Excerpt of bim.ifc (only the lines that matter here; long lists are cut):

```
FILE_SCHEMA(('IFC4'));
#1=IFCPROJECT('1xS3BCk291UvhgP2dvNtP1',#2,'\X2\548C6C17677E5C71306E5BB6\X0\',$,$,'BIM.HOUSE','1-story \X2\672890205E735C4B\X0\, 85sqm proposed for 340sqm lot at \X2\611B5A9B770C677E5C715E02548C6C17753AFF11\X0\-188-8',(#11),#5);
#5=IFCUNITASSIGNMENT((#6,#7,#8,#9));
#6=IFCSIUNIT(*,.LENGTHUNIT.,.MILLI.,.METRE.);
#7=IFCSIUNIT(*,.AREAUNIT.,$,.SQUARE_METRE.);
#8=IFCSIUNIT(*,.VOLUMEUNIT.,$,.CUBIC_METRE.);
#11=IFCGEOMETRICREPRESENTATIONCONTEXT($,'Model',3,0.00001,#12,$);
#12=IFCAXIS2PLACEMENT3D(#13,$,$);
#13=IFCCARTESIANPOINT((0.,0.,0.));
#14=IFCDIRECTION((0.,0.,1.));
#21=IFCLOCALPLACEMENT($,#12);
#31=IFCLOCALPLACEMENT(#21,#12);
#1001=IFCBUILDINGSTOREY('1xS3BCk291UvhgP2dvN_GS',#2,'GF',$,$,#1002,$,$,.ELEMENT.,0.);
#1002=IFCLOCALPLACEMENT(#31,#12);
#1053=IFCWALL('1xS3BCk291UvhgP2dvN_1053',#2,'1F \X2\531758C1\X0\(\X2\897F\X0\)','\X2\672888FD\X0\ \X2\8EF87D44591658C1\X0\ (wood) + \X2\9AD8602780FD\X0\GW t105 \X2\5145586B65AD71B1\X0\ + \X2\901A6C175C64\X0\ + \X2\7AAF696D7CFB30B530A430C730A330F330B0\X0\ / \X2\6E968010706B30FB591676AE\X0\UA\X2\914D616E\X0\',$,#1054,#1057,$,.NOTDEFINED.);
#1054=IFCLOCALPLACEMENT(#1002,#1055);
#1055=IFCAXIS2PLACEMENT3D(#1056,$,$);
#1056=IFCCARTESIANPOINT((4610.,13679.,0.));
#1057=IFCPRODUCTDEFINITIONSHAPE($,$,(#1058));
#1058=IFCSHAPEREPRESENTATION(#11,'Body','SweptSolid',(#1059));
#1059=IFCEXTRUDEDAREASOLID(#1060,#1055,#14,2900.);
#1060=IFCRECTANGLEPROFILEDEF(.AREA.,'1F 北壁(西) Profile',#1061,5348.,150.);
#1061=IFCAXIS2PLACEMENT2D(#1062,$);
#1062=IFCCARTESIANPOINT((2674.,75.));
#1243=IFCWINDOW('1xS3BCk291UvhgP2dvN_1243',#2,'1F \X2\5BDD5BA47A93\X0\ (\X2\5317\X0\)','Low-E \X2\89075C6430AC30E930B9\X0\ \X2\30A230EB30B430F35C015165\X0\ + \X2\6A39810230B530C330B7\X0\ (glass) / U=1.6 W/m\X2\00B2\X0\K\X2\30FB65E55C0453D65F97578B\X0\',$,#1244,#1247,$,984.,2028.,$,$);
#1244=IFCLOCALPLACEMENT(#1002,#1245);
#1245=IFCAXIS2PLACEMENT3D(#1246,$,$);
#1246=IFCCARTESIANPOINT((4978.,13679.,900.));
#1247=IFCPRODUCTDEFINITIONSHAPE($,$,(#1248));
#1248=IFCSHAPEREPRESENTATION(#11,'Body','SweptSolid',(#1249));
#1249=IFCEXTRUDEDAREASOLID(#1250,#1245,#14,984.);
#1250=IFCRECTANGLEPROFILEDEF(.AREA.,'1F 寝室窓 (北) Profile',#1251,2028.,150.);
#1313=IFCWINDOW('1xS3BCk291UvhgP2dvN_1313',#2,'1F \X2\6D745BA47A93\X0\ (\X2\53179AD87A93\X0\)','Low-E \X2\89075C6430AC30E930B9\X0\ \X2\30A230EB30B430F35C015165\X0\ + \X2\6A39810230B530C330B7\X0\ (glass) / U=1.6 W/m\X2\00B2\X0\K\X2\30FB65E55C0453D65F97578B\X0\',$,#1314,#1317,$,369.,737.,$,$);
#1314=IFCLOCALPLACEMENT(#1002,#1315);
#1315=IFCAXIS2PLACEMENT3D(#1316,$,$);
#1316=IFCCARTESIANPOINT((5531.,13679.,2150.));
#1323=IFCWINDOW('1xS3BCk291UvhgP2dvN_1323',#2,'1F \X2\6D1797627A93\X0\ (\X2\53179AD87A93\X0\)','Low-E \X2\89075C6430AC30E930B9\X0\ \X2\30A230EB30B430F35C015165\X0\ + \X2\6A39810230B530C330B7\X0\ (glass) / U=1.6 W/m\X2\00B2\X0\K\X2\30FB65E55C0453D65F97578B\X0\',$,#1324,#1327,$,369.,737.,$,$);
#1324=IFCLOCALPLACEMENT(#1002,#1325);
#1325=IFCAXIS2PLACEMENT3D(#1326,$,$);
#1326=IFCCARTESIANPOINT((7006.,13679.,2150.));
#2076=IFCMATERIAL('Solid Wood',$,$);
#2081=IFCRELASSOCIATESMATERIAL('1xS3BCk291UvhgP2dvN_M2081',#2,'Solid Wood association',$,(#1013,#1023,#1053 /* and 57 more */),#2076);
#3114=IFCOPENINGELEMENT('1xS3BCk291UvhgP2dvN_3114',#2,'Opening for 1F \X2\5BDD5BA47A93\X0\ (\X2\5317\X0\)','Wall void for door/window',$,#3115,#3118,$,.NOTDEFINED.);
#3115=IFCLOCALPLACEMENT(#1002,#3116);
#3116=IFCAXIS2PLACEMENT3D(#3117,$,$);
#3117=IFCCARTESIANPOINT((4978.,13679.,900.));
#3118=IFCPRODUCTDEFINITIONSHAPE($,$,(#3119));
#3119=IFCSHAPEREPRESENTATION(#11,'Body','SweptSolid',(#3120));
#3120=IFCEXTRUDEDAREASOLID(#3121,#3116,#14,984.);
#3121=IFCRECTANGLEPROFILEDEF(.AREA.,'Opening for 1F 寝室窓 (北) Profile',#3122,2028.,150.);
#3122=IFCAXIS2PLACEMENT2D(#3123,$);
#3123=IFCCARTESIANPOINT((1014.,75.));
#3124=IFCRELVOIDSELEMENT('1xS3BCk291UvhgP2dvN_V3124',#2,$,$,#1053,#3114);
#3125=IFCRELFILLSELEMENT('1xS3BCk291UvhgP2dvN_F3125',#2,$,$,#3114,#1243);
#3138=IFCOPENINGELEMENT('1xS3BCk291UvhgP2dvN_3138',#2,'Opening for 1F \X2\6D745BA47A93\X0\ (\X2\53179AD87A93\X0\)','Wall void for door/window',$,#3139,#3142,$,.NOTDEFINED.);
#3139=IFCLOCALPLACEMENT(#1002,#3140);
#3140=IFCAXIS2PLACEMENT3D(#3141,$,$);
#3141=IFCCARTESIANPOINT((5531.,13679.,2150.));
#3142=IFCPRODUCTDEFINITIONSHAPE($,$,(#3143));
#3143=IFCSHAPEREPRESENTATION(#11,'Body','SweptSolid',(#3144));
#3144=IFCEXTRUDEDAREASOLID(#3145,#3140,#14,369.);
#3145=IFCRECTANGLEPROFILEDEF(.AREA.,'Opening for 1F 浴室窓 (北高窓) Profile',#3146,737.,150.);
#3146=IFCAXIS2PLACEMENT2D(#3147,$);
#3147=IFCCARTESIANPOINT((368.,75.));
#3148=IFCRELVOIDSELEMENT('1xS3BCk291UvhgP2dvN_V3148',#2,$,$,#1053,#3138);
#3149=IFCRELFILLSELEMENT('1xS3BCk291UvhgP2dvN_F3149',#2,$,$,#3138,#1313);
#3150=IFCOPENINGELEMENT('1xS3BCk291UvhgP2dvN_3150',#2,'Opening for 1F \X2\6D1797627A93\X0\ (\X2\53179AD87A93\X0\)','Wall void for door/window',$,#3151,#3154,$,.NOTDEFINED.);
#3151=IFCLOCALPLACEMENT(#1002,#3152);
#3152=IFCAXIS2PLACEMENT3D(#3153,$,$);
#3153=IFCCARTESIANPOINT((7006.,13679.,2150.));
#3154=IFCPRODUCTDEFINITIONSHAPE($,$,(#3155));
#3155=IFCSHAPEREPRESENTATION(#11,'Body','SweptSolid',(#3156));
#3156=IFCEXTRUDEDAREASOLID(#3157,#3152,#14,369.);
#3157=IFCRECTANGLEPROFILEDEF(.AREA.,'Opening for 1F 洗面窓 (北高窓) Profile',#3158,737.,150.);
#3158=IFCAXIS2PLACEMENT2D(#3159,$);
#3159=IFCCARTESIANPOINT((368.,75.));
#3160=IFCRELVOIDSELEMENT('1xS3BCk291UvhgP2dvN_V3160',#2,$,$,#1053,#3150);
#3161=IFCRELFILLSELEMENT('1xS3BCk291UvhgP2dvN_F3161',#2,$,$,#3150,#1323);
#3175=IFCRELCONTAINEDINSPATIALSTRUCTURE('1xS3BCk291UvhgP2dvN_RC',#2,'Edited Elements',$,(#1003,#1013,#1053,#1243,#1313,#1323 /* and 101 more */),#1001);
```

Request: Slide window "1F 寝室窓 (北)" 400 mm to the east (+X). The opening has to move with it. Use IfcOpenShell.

```python
import ifcopenshell
import ifcopenshell.api.geometry
import ifcopenshell.util.placement
import ifcopenshell.util.unit

model = ifcopenshell.open("bim.ifc")
unit_scale = ifcopenshell.util.unit.calculate_unit_scale(model)

window = model.by_id(1243)
opening = window.FillsVoids[0].RelatingOpeningElement
wall = opening.VoidsElements[0].RelatingBuildingElement

wall_matrix = ifcopenshell.util.placement.get_local_placement(wall.ObjectPlacement)
shift = wall_matrix[:3, 0] * 0.4 / unit_scale
before = ifcopenshell.util.placement.get_local_placement(window.ObjectPlacement)[:3, 3].copy()

# The window is not placed relative to its opening, so move both.
for product in (opening, window):
    matrix = ifcopenshell.util.placement.get_local_placement(product.ObjectPlacement)
    matrix[:3, 3] += shift
    ifcopenshell.api.geometry.edit_object_placement(model, product=product, matrix=matrix, is_si=False)

after = ifcopenshell.util.placement.get_local_placement(window.ObjectPlacement)[:3, 3]
print("window moved by", (after - before).round(3) + 0.0)

model.write("bim_edited.ifc")
```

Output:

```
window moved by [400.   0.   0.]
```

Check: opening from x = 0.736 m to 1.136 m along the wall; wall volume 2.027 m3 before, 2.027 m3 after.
